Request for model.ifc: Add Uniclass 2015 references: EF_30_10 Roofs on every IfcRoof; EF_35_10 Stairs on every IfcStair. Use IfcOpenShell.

First a look at what the model holds.

```python
import ifcopenshell

model = ifcopenshell.open("model.ifc")
print(model.schema)
print("classifications:", [c.Name for c in model.by_type("IfcClassification")])
for ifc_class in ("IfcDoor", "IfcRoof", "IfcStair", "IfcWall", "IfcWindow"):
    print(ifc_class, len(model.by_type(ifc_class)))
```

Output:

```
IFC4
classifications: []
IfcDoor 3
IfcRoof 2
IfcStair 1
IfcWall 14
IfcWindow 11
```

```python
import ifcopenshell
import ifcopenshell.api.classification

model = ifcopenshell.open("model.ifc")

system = ifcopenshell.api.classification.add_classification(model, classification="Uniclass 2015")

codes = {
    "IfcRoof": ("EF_30_10", "Roofs"),
    "IfcStair": ("EF_35_10", "Stairs"),
}
for ifc_class, (code, name) in codes.items():
    products = model.by_type(ifc_class)
    ifcopenshell.api.classification.add_reference(
        model, products=products, classification=system, identification=code, name=name
    )
    print(code, len(products))

model.write("model_edited.ifc")
```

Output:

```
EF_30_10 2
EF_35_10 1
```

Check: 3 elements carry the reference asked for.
